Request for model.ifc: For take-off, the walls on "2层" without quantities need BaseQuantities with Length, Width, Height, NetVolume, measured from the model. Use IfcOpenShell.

First a look at what the model holds.

```python
import ifcopenshell
import ifcopenshell.util.element
import ifcopenshell.util.unit

model = ifcopenshell.open("model.ifc")
print(model.schema)
for unit_type in ("LENGTHUNIT", "AREAUNIT", "VOLUMEUNIT"):
    print(unit_type, ifcopenshell.util.unit.calculate_unit_scale(model, unit_type))
storey = next(s for s in model.by_type("IfcBuildingStorey") if s.Name == "2层")
walls = [e for e in ifcopenshell.util.element.get_decomposition(storey) if e.is_a("IfcWall")]
for e in sorted(walls, key=lambda e: e.id()):
    print(e.id(), e.is_a(), e.Name, list(ifcopenshell.util.element.get_psets(e, qtos_only=True)), sep=" | ")
```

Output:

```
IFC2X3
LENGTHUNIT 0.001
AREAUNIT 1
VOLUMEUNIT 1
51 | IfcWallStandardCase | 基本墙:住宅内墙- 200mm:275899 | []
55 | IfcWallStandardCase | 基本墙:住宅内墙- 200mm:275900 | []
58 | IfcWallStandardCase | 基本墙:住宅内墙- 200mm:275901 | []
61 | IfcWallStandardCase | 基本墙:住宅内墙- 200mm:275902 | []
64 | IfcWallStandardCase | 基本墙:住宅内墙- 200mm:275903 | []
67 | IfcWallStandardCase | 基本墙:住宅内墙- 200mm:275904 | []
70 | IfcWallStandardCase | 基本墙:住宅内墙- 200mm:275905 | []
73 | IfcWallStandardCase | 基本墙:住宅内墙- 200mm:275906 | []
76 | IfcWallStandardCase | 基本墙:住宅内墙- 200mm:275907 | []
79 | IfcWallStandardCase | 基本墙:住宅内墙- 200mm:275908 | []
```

```python
import ifcopenshell
import ifcopenshell.api.pset
import ifcopenshell.geom
import ifcopenshell.util.element
import ifcopenshell.util.shape
import ifcopenshell.util.unit

model = ifcopenshell.open("model.ifc")
unit_scale = ifcopenshell.util.unit.calculate_unit_scale(model)
volume_scale = ifcopenshell.util.unit.calculate_unit_scale(model, "VOLUMEUNIT")
settings = ifcopenshell.geom.settings()

storey = next(s for s in model.by_type("IfcBuildingStorey") if s.Name == "2层")
walls = [e for e in ifcopenshell.util.element.get_decomposition(storey) if e.is_a("IfcWall")]

for e in sorted(walls, key=lambda e: e.id()):
    if ifcopenshell.util.element.get_psets(e, qtos_only=True, should_inherit=False):
        continue
    # Geometry comes back in metres, in the element's own axes.
    shape = ifcopenshell.geom.create_shape(settings, e)
    values = {
        "Length": ifcopenshell.util.shape.get_x(shape.geometry) / unit_scale,
        "Width": ifcopenshell.util.shape.get_y(shape.geometry) / unit_scale,
        "Height": ifcopenshell.util.shape.get_z(shape.geometry) / unit_scale,
        "NetVolume": ifcopenshell.util.shape.get_volume(shape.geometry) / volume_scale,
    }
    qto = ifcopenshell.api.pset.add_qto(model, product=e, name="BaseQuantities")
    ifcopenshell.api.pset.edit_qto(model, qto=qto, properties=values)
    print(e.id(), {k: round(v, 3) for k, v in values.items()})

model.write("model_updated.ifc")
```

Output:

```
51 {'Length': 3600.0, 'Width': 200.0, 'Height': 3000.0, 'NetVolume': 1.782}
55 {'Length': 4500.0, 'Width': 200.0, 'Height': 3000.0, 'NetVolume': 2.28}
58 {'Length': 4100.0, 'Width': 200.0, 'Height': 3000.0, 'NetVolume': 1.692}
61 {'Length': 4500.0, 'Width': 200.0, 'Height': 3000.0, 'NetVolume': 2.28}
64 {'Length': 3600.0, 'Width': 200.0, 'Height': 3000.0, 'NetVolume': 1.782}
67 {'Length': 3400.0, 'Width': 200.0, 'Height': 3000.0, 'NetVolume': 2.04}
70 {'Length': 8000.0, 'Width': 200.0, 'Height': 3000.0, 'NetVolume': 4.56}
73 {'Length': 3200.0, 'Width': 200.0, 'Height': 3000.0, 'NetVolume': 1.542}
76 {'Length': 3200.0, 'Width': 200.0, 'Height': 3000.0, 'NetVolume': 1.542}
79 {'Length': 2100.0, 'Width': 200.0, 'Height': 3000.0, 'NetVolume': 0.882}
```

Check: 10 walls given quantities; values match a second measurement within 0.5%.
